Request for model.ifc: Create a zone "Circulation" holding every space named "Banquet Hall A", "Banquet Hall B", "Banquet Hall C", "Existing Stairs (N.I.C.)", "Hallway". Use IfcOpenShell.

First a look at what the model holds.

```python
import ifcopenshell

model = ifcopenshell.open("model.ifc")
print(model.schema)
seen = {}
for space in model.by_type("IfcSpace"):
    seen[space.LongName] = seen.get(space.LongName, 0) + 1
for name, count in sorted(seen.items(), key=str):
    print(count, "x", name)
print("zones:", [z.Name for z in model.by_type("IfcZone")][:20])
```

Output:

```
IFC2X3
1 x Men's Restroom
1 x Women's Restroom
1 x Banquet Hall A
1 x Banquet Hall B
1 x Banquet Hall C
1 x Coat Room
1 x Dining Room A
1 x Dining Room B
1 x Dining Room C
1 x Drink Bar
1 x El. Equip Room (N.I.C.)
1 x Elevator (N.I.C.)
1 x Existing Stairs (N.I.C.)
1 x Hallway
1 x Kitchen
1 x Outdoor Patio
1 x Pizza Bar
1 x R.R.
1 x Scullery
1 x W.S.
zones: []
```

```python
import ifcopenshell
import ifcopenshell.api.group
import ifcopenshell.api.root

model = ifcopenshell.open("model.ifc")

names = {"Banquet Hall A", "Banquet Hall B", "Banquet Hall C", "Existing Stairs (N.I.C.)", "Hallway"}
spaces = [s for s in model.by_type("IfcSpace") if s.LongName in names]

zone = ifcopenshell.api.root.create_entity(model, ifc_class="IfcZone", name="Circulation")
ifcopenshell.api.group.assign_group(model, products=spaces, group=zone)
print(len(spaces), "spaces in", zone.Name)

model.write("model_rev.ifc")
```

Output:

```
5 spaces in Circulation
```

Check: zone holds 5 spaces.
